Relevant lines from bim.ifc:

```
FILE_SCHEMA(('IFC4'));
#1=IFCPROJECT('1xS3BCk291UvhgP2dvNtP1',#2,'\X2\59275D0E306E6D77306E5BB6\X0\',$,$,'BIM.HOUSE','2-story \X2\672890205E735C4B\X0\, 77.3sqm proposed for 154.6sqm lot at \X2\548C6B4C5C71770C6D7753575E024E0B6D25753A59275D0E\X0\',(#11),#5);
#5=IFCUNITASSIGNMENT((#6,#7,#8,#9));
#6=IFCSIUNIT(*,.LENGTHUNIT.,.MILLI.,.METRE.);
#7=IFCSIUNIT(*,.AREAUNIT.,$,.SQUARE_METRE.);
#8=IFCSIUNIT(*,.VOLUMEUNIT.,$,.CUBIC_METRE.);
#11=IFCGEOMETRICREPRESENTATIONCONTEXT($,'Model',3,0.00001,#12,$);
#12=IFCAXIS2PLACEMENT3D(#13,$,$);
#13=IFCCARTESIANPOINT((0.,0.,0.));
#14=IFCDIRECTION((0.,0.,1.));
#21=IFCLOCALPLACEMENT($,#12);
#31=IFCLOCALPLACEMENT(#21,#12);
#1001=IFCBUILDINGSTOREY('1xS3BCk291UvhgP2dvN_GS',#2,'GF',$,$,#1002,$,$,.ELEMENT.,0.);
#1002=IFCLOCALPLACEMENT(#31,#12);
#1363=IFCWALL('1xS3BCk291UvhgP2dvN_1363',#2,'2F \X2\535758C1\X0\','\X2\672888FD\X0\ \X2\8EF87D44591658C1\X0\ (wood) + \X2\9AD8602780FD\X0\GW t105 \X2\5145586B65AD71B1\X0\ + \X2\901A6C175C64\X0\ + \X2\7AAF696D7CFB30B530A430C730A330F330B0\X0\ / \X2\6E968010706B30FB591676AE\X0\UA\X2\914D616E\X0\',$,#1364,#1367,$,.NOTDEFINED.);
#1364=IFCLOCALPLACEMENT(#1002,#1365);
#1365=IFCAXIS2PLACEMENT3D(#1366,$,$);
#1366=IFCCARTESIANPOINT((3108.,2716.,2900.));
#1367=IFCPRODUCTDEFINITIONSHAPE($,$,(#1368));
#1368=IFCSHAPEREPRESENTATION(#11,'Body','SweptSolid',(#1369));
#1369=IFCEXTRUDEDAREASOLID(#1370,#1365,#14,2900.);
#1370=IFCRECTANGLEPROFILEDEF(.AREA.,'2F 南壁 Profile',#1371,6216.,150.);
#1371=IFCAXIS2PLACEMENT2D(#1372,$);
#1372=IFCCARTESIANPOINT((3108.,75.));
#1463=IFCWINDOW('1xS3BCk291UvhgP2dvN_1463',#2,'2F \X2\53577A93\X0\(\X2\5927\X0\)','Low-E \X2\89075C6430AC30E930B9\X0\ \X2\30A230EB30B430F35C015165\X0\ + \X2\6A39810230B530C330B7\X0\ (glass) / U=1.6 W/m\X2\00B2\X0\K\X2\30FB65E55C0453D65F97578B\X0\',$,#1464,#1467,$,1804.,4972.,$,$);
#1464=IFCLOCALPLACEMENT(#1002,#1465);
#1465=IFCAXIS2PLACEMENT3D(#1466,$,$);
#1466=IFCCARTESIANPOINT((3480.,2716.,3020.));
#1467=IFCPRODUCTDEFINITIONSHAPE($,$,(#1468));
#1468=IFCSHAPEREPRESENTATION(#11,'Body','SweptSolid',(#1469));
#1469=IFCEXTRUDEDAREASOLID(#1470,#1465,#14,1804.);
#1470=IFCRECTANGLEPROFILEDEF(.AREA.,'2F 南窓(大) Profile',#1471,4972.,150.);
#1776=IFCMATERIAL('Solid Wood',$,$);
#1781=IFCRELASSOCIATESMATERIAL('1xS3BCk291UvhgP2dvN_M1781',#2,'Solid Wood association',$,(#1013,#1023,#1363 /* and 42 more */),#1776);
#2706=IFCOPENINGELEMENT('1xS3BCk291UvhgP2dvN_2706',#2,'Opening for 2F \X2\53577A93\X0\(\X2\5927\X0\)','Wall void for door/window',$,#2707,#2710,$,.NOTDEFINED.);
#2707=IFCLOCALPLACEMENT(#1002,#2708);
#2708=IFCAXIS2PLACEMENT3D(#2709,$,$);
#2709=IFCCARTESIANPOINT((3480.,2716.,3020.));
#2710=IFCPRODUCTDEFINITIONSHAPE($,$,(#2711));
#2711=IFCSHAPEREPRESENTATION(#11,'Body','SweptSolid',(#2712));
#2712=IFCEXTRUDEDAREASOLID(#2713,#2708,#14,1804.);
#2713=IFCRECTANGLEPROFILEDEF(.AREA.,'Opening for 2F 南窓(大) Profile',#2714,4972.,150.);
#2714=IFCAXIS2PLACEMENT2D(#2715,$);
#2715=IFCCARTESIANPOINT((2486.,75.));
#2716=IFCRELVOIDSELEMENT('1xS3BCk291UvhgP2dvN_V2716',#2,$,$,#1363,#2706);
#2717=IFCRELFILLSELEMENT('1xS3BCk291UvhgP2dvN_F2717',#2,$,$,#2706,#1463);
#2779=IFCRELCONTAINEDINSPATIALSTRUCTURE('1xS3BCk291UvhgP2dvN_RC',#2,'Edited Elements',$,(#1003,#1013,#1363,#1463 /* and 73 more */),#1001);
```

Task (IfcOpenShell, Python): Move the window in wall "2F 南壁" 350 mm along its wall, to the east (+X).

```python
import ifcopenshell
import ifcopenshell.api.geometry
import ifcopenshell.util.placement

model = ifcopenshell.open("bim.ifc")

window = model.by_guid("1xS3BCk291UvhgP2dvN_1463")
opening = window.FillsVoids[0].RelatingOpeningElement
wall = opening.VoidsElements[0].RelatingBuildingElement

wall_matrix = ifcopenshell.util.placement.get_local_placement(wall.ObjectPlacement)
shift = wall_matrix[:3, 0] * 350.0
before = ifcopenshell.util.placement.get_local_placement(window.ObjectPlacement)[:3, 3].copy()

# The window is not placed relative to its opening, so move both.
for product in (opening, window):
    matrix = ifcopenshell.util.placement.get_local_placement(product.ObjectPlacement)
    matrix[:3, 3] += shift
    ifcopenshell.api.geometry.edit_object_placement(model, product=product, matrix=matrix, is_si=False)

after = ifcopenshell.util.placement.get_local_placement(window.ObjectPlacement)[:3, 3]
print("window moved by", (after - before).round(3) + 0.0)

model.write("bim_updated.ifc")
```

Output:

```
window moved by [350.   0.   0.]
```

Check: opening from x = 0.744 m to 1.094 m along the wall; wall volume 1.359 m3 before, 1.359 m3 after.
